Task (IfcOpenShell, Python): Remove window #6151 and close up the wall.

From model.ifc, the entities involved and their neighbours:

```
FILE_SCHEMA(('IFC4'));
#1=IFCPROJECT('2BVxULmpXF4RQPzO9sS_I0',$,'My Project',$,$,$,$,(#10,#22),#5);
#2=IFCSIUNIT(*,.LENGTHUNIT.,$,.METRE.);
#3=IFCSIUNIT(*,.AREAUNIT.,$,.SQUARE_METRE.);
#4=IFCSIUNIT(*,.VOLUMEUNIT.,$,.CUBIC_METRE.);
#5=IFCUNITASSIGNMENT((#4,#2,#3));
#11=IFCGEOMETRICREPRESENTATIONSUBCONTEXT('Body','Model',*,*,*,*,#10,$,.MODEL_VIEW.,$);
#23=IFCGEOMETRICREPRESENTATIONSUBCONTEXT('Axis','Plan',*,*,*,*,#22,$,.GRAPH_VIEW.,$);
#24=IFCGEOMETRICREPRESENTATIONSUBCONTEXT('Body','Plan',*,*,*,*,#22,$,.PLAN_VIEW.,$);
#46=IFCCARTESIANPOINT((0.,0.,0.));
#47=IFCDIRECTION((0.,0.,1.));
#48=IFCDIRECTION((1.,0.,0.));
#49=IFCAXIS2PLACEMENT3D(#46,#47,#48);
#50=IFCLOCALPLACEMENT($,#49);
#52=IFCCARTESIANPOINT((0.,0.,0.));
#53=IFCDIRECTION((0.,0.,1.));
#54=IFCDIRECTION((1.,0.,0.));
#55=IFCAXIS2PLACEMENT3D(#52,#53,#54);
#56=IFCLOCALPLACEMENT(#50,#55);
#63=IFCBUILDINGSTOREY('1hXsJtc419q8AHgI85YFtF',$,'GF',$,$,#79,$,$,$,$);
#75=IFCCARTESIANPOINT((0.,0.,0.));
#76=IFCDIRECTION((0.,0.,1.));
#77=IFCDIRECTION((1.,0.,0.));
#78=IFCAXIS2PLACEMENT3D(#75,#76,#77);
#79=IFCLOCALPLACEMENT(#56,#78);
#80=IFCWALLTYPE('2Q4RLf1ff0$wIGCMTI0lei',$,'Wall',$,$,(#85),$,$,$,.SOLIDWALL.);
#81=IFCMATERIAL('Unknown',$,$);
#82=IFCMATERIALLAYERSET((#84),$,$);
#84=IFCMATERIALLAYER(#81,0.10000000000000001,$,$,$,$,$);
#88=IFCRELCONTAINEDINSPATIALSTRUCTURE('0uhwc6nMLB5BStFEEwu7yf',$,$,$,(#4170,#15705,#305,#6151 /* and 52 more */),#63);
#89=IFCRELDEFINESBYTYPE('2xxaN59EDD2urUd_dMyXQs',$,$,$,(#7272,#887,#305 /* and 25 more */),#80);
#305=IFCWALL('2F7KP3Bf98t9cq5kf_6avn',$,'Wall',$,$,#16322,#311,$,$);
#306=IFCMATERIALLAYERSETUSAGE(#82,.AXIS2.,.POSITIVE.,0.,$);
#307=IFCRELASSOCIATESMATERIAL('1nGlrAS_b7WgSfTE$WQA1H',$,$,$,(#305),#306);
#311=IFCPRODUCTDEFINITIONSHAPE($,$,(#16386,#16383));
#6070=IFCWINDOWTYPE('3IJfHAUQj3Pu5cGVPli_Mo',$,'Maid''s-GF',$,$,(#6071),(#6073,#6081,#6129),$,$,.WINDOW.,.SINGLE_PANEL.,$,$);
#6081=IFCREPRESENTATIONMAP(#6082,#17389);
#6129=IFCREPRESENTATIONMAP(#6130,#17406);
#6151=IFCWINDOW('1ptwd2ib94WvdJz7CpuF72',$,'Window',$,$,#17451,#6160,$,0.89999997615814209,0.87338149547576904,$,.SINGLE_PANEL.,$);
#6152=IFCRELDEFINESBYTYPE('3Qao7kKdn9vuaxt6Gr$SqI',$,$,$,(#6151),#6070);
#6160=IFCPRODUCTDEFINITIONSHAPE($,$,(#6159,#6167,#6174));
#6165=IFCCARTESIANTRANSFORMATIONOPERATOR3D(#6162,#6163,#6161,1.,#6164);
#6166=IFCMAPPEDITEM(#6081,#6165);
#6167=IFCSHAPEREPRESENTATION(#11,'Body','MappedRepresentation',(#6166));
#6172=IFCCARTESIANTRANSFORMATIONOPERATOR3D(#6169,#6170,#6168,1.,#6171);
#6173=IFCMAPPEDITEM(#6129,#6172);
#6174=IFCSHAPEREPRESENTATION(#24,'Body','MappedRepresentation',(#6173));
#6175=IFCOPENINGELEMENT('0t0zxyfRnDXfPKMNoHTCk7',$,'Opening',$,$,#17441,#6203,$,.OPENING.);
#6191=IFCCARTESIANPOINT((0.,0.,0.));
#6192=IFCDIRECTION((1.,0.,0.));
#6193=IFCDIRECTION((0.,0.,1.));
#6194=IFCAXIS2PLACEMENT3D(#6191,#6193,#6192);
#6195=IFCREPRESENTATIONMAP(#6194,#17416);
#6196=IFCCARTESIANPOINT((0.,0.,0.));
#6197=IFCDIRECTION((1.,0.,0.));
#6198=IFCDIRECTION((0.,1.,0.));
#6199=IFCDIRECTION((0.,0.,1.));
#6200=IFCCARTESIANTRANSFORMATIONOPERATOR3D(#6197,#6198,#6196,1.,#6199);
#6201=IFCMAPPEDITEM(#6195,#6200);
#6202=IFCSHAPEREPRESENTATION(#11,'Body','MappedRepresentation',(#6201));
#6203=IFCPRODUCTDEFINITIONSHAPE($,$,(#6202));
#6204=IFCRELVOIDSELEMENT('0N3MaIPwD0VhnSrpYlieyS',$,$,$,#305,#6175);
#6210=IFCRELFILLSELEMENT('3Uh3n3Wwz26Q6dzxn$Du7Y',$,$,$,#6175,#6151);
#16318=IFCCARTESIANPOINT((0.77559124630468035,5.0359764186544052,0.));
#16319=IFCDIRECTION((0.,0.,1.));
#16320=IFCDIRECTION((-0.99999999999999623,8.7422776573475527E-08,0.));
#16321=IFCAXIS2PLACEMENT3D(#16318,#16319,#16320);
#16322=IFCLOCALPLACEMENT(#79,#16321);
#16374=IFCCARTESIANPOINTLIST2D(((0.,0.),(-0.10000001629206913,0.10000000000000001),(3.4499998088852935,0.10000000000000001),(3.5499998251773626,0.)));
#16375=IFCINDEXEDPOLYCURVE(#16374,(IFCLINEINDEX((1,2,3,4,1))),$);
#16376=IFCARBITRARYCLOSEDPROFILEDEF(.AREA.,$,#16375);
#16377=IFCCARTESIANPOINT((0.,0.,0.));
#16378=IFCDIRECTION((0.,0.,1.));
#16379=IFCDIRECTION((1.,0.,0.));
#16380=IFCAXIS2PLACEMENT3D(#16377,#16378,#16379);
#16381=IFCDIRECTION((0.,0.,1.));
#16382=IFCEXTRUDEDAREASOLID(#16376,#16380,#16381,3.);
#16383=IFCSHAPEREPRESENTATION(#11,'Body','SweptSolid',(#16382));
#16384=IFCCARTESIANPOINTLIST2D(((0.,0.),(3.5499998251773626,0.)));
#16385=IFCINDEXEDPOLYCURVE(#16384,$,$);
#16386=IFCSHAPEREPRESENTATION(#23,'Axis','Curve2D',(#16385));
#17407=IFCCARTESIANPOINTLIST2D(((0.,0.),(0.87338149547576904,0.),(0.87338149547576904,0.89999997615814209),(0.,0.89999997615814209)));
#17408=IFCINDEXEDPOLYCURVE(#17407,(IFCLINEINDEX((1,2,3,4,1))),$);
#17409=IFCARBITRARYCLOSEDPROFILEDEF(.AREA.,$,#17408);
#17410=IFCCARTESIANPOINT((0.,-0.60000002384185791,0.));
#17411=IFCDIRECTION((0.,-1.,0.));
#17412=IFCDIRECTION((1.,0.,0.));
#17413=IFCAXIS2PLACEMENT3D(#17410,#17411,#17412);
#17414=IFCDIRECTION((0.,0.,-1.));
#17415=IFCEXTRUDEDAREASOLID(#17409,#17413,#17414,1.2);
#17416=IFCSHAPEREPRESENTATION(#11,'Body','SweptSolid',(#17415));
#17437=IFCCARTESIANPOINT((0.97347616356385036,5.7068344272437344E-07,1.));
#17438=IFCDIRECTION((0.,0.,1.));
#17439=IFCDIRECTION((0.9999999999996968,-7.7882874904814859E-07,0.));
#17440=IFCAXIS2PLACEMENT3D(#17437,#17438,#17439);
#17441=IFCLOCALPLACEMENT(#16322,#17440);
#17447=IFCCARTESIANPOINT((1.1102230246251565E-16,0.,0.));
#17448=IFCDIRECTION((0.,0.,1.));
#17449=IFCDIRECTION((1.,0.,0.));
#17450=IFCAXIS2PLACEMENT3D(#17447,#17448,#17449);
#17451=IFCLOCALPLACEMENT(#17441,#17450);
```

```python
import ifcopenshell
import ifcopenshell.api.feature
import ifcopenshell.api.root
import ifcopenshell.geom
import ifcopenshell.util.shape

model = ifcopenshell.open("model.ifc")
settings = ifcopenshell.geom.settings()


def volume(element):
    """Net volume in cubic metres, openings subtracted."""
    shape = ifcopenshell.geom.create_shape(settings, element)
    return ifcopenshell.util.shape.get_volume(shape.geometry)


window = model.by_guid("1ptwd2ib94WvdJz7CpuF72")
opening = window.FillsVoids[0].RelatingOpeningElement
wall = opening.VoidsElements[0].RelatingBuildingElement
before = volume(wall)

ifcopenshell.api.root.remove_product(model, product=window)
ifcopenshell.api.feature.remove_feature(model, feature=opening)

after = volume(wall)

print(f"wall volume {before:.3f} -> {after:.3f} m3")

model.write("model-out.ifc")
```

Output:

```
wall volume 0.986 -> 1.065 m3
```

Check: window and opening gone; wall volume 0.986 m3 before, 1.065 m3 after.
